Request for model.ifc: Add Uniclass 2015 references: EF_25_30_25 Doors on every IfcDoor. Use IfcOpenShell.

First a look at what the model holds.

```python
import ifcopenshell

model = ifcopenshell.open("model.ifc")
print(model.schema)
print("classifications:", [c.Name for c in model.by_type("IfcClassification")])
for ifc_class in ("IfcDoor", "IfcRoof", "IfcStair", "IfcWall", "IfcWindow"):
    print(ifc_class, len(model.by_type(ifc_class)))
```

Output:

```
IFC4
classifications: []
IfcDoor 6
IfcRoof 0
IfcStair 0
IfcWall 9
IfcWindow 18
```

```python
import ifcopenshell
import ifcopenshell.api.classification

model = ifcopenshell.open("model.ifc")

system = ifcopenshell.api.classification.add_classification(model, classification="Uniclass 2015")

codes = {
    "IfcDoor": ("EF_25_30_25", "Doors"),
}
for ifc_class, (code, name) in codes.items():
    products = model.by_type(ifc_class)
    ifcopenshell.api.classification.add_reference(
        model, products=products, classification=system, identification=code, name=name
    )
    print(code, len(products))

model.write("model_rev.ifc")
```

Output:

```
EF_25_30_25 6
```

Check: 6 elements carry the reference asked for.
